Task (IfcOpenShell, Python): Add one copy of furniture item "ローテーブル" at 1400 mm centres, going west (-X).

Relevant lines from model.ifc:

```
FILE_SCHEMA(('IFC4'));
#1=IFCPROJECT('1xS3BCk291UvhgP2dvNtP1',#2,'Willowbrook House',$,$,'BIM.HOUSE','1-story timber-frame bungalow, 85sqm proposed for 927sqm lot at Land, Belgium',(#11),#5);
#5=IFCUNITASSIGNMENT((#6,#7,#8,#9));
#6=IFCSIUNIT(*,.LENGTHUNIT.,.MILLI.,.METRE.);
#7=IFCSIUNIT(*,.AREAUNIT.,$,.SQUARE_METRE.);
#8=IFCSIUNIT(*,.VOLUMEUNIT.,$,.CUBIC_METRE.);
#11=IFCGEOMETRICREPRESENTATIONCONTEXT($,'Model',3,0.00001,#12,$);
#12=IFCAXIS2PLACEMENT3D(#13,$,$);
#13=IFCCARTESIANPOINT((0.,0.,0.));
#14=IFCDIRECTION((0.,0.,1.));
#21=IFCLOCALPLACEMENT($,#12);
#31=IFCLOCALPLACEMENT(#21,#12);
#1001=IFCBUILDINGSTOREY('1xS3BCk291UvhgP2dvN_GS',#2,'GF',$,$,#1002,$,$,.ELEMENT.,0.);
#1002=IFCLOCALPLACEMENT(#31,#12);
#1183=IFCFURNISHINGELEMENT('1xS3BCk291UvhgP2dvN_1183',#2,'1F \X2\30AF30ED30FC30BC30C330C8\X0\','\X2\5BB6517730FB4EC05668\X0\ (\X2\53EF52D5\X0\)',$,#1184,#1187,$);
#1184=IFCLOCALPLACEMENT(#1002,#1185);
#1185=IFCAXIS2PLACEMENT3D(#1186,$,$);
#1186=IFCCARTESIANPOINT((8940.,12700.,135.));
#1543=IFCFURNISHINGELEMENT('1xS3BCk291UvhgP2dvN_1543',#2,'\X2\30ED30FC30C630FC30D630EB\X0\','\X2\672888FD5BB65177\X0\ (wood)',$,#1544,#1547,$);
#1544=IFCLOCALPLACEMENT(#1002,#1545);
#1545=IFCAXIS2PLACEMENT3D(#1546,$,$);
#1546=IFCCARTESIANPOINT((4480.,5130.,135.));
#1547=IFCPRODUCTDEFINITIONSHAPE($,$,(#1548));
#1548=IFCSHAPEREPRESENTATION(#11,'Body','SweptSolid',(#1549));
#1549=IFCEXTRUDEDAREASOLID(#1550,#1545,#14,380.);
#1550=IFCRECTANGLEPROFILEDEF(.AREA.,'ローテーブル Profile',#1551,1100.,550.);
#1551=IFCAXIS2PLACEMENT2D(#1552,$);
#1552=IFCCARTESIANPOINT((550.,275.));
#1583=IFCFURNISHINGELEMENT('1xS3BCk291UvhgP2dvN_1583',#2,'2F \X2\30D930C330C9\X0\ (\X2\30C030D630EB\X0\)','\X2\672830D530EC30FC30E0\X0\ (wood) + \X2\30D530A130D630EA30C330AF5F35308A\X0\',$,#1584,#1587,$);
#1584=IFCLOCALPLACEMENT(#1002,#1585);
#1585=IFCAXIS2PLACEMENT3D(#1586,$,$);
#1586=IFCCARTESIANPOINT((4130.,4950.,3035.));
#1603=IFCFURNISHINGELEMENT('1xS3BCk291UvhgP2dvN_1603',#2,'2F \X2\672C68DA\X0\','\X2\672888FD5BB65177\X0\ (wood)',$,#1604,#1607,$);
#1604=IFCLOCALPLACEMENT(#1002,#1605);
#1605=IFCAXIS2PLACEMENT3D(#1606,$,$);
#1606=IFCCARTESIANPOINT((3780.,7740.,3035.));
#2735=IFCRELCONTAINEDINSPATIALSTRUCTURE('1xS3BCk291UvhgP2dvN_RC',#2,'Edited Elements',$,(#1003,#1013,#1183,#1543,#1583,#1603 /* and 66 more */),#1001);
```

```python
import numpy as np
import ifcopenshell
import ifcopenshell.api.geometry
import ifcopenshell.api.root
import ifcopenshell.util.element
import ifcopenshell.util.placement
import ifcopenshell.util.unit

model = ifcopenshell.open("model.ifc")
unit_scale = ifcopenshell.util.unit.calculate_unit_scale(model)


def reuse_history(source, copy):
    """copy_class also copies each property set's owner history, people and application; keep the originals."""
    for rel in copy.IsDefinedBy:
        if rel.is_a("IfcRelDefinesByProperties") and (history := rel.RelatingPropertyDefinition.OwnerHistory):
            rel.RelatingPropertyDefinition.OwnerHistory = source.OwnerHistory
            ifcopenshell.util.element.remove_deep2(model, history)


source = model.by_id(1543)
base = ifcopenshell.util.placement.get_local_placement(source.ObjectPlacement)
step = np.array([-1.0, 0.0, 0.0]) * 1.4 / unit_scale

for i in range(1, 2):
    copy = ifcopenshell.api.root.copy_class(model, product=source)
    copy.Representation = ifcopenshell.util.element.copy_deep(
        model, source.Representation, exclude=["IfcGeometricRepresentationContext", "IfcRepresentationMap"]
    )
    reuse_history(source, copy)
    matrix = base.copy()
    matrix[:3, 3] += i * step
    print("added at", matrix[:3, 3].round(3) + 0.0)
    ifcopenshell.api.geometry.edit_object_placement(model, product=copy, matrix=matrix, is_si=False)

model.write("model_updated.ifc")
```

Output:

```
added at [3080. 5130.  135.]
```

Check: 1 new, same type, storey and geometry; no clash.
